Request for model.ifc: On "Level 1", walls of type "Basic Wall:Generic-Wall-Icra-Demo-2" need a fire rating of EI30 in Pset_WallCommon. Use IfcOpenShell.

First a look at what the model holds.

```python
import ifcopenshell
import ifcopenshell.util.element

model = ifcopenshell.open("model.ifc")
print(model.schema)
storey = next(s for s in model.by_type("IfcBuildingStorey") if s.Name == "Level 1")
walls = [e for e in ifcopenshell.util.element.get_decomposition(storey) if e.is_a("IfcWall")]
seen = {}
for e in walls:
    element_type = ifcopenshell.util.element.get_type(e)
    key = (element_type.Name if element_type != e and element_type else None, ifcopenshell.util.element.get_pset(e, "Pset_WallCommon", "FireRating"))
    seen[key] = seen.get(key, 0) + 1
for (name, value), count in sorted(seen.items(), key=str):
    print(count, "x", name, "|", value)
```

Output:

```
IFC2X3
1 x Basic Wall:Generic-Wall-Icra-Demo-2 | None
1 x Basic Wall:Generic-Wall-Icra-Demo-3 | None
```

```python
import ifcopenshell
import ifcopenshell.api.pset
import ifcopenshell.util.element

model = ifcopenshell.open("model.ifc")

storey = next(s for s in model.by_type("IfcBuildingStorey") if s.Name == "Level 1")
walls = [e for e in ifcopenshell.util.element.get_decomposition(storey) if e.is_a("IfcWall")]

count = 0
for e in walls:
    element_type = ifcopenshell.util.element.get_type(e)
    if element_type in (None, e) or element_type.Name != "Basic Wall:Generic-Wall-Icra-Demo-2":
        continue
    # add_pset returns the element's existing set when there is one.
    pset = ifcopenshell.api.pset.add_pset(model, product=e, name="Pset_WallCommon")
    ifcopenshell.api.pset.edit_pset(model, pset=pset, properties={"FireRating": "EI30"})
    count += 1

print(count, "walls updated")

model.write("model_v2.ifc")
```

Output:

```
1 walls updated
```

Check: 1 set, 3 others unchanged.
